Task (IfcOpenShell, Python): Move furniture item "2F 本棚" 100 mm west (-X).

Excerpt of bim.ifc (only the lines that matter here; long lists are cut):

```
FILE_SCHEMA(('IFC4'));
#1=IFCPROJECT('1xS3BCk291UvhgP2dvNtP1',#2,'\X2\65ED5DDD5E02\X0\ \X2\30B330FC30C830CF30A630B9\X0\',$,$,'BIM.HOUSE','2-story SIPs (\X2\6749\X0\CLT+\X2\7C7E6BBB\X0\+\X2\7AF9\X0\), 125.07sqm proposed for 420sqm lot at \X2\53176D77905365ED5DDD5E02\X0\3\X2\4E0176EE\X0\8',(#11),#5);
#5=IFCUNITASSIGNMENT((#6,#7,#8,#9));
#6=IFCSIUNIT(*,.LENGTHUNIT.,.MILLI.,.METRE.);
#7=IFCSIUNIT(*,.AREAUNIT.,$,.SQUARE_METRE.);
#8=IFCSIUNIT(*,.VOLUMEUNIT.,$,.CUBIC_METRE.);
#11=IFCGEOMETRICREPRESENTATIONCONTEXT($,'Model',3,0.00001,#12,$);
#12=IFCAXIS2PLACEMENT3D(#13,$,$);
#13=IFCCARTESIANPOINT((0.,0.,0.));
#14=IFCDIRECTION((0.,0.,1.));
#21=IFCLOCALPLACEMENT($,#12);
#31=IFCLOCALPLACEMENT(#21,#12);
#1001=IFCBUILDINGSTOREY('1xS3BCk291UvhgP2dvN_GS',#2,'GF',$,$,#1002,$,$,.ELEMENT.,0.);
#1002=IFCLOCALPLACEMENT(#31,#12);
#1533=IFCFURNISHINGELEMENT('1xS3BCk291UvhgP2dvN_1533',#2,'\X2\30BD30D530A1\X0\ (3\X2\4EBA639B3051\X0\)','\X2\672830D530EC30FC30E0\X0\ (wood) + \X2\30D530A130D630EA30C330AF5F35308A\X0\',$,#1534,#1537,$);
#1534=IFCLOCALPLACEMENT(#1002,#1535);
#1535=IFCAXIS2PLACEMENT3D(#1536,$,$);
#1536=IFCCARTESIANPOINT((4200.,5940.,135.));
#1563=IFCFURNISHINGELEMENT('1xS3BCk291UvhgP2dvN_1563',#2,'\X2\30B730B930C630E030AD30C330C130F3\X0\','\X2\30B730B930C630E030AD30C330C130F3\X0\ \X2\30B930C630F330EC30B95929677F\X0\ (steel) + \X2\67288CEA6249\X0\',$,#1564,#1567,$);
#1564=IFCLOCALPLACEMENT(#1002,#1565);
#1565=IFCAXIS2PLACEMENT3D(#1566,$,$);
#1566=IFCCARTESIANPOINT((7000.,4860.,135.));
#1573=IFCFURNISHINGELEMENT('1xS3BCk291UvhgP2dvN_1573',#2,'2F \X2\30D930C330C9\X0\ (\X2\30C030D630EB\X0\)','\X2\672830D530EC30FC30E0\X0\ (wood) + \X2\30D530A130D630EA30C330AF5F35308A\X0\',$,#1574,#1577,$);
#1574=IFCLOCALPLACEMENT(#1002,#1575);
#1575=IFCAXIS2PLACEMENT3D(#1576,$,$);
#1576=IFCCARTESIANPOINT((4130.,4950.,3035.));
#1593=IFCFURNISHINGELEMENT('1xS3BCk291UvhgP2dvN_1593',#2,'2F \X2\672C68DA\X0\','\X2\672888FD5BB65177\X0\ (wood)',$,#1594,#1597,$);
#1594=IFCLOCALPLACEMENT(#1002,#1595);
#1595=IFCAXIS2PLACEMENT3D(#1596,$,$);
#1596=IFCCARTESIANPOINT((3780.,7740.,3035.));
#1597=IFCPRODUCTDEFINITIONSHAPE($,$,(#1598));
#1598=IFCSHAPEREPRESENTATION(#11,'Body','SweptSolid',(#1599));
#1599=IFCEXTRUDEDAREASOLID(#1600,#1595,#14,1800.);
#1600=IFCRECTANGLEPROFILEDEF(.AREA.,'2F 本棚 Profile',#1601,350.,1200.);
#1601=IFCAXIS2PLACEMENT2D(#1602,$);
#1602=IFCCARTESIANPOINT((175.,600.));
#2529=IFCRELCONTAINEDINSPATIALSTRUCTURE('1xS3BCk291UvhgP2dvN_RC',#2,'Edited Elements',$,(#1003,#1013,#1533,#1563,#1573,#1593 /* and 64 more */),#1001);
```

```python
import ifcopenshell
import ifcopenshell.api.geometry
import ifcopenshell.util.placement
import ifcopenshell.util.unit

model = ifcopenshell.open("bim.ifc")
unit_scale = ifcopenshell.util.unit.calculate_unit_scale(model)

item = model.by_guid("1xS3BCk291UvhgP2dvN_1593")
matrix = ifcopenshell.util.placement.get_local_placement(item.ObjectPlacement)
matrix[0, 3] -= 0.1 / unit_scale
ifcopenshell.api.geometry.edit_object_placement(model, product=item, matrix=matrix, is_si=False)

print(ifcopenshell.util.placement.get_local_placement(item.ObjectPlacement).round(3) + 0.0)

model.write("bim_edited.ifc")
```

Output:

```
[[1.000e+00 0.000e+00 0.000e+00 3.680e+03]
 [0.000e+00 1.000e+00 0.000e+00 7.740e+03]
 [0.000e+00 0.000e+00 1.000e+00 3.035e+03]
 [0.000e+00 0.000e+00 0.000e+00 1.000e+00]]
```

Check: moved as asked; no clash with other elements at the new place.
